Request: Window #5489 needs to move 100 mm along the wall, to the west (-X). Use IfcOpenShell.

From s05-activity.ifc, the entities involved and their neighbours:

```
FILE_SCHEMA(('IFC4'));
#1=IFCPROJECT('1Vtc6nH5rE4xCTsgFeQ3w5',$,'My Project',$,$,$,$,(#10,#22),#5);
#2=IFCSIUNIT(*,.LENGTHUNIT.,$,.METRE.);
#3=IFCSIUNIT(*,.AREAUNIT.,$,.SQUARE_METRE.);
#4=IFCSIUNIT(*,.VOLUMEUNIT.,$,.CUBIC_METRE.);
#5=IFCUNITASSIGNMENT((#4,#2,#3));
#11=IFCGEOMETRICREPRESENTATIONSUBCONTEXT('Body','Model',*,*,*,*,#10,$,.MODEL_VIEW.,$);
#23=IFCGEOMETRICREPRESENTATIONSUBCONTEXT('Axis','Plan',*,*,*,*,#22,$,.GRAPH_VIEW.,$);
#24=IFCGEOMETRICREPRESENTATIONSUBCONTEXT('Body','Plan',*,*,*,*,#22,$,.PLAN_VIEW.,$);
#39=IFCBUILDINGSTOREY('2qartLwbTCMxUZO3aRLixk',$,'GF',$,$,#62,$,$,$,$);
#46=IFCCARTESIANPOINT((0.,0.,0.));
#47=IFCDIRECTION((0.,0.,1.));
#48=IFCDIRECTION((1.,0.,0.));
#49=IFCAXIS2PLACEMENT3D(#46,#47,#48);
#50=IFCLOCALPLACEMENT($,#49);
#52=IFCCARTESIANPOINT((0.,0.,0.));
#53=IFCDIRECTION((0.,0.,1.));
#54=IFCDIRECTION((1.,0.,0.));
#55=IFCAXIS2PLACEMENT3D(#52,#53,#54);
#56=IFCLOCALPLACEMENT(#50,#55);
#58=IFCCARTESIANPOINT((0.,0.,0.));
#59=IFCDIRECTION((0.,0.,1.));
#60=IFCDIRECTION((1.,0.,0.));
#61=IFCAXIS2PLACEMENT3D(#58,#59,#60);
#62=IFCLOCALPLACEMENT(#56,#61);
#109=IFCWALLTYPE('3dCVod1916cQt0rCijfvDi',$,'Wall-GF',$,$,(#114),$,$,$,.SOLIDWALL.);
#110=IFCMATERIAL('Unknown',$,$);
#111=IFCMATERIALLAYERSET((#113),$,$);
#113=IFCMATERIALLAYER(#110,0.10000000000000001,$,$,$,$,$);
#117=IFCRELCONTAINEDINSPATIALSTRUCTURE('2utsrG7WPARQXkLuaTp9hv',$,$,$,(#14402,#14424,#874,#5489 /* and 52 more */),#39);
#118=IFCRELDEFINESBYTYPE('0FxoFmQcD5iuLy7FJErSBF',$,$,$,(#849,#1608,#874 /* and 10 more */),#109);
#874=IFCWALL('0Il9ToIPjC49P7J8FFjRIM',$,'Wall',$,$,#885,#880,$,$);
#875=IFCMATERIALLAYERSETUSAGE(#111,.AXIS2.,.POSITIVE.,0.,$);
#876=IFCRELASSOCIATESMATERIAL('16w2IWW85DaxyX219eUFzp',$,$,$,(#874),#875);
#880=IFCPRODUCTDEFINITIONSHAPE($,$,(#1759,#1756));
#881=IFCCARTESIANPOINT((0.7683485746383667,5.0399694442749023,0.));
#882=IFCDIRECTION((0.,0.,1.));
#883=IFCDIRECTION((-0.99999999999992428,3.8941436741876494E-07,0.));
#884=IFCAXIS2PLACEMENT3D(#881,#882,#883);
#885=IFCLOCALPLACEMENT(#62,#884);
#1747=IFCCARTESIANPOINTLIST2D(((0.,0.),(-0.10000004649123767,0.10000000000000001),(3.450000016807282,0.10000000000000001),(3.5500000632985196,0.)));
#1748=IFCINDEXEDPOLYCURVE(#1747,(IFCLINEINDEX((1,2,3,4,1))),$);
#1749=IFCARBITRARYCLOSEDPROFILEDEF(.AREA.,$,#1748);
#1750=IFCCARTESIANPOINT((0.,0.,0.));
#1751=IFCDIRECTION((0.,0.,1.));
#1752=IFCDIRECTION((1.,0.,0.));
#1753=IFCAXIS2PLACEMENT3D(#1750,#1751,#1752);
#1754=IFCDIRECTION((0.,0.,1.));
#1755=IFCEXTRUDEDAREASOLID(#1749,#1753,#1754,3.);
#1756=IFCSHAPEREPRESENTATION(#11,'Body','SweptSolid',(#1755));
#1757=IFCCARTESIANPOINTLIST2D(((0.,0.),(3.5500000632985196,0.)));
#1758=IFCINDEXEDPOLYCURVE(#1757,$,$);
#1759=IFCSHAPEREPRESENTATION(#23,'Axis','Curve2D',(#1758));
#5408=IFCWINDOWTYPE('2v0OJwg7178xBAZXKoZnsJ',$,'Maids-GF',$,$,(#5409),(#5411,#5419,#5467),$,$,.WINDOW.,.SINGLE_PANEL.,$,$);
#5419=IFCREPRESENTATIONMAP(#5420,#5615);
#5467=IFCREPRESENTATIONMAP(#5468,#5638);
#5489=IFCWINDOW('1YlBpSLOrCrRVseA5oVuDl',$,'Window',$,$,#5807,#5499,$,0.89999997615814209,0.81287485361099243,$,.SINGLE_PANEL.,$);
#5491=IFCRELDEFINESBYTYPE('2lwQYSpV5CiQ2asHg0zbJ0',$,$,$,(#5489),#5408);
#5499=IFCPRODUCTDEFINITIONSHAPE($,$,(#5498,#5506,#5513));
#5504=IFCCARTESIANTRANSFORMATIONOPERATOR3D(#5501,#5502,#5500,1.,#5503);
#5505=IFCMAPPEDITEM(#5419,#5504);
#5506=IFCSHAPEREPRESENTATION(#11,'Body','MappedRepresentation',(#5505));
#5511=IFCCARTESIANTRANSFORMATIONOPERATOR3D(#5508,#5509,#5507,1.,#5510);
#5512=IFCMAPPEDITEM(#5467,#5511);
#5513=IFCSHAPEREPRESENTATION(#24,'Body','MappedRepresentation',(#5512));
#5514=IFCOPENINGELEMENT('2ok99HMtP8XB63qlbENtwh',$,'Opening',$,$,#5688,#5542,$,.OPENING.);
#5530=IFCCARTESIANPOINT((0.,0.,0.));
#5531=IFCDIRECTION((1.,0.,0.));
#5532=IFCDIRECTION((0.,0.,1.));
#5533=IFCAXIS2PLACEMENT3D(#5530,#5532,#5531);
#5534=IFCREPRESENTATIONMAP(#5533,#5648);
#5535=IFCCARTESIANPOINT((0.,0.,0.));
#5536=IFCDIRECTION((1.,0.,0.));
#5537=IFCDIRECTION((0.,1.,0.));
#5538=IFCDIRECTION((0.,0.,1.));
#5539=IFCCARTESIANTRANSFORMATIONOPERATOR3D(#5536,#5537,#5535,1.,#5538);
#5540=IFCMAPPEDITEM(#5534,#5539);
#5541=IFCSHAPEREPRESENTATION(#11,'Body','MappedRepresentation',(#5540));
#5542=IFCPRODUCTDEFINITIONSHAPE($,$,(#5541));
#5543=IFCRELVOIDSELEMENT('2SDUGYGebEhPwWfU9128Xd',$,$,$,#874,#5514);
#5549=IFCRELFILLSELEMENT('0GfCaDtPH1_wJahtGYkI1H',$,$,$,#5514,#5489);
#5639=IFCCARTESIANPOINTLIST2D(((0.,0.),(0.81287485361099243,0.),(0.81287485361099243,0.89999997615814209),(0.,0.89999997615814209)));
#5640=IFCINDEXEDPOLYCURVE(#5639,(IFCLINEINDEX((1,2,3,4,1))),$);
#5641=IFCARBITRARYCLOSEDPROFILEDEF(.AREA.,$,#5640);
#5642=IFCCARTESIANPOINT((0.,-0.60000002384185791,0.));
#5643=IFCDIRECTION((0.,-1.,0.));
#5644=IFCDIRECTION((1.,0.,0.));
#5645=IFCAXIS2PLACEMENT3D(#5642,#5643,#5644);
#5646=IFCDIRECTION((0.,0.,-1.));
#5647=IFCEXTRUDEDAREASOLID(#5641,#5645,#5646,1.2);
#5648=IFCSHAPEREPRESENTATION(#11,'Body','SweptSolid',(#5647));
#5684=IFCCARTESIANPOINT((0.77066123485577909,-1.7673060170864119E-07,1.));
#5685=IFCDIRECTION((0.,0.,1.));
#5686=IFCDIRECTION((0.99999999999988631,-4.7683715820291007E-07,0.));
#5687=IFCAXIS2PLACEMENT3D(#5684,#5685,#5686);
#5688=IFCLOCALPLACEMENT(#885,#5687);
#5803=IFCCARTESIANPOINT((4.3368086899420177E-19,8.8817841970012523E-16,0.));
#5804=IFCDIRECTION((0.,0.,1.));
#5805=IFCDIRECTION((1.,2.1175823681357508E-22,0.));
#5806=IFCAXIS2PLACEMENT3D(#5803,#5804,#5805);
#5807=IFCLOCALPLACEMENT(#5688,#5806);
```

```python
import ifcopenshell
import ifcopenshell.api.geometry
import ifcopenshell.util.placement
import ifcopenshell.util.unit

model = ifcopenshell.open("s05-activity.ifc")
unit_scale = ifcopenshell.util.unit.calculate_unit_scale(model)

window = model.by_guid("1YlBpSLOrCrRVseA5oVuDl")
opening = window.FillsVoids[0].RelatingOpeningElement
wall = opening.VoidsElements[0].RelatingBuildingElement

wall_matrix = ifcopenshell.util.placement.get_local_placement(wall.ObjectPlacement)
shift = wall_matrix[:3, 0] * 0.1 / unit_scale
before = ifcopenshell.util.placement.get_local_placement(window.ObjectPlacement)[:3, 3].copy()

# The window is placed relative to its opening, so it follows when the opening moves.
matrix = ifcopenshell.util.placement.get_local_placement(opening.ObjectPlacement)
matrix[:3, 3] += shift
ifcopenshell.api.geometry.edit_object_placement(
    model, product=opening, matrix=matrix, is_si=False, should_transform_children=True
)

after = ifcopenshell.util.placement.get_local_placement(window.ObjectPlacement)[:3, 3]
print("window moved by", (after - before).round(3) + 0.0)

model.write("s05-activity_v2.ifc")
```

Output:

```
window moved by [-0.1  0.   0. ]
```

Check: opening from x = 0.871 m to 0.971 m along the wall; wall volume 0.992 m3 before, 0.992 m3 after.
